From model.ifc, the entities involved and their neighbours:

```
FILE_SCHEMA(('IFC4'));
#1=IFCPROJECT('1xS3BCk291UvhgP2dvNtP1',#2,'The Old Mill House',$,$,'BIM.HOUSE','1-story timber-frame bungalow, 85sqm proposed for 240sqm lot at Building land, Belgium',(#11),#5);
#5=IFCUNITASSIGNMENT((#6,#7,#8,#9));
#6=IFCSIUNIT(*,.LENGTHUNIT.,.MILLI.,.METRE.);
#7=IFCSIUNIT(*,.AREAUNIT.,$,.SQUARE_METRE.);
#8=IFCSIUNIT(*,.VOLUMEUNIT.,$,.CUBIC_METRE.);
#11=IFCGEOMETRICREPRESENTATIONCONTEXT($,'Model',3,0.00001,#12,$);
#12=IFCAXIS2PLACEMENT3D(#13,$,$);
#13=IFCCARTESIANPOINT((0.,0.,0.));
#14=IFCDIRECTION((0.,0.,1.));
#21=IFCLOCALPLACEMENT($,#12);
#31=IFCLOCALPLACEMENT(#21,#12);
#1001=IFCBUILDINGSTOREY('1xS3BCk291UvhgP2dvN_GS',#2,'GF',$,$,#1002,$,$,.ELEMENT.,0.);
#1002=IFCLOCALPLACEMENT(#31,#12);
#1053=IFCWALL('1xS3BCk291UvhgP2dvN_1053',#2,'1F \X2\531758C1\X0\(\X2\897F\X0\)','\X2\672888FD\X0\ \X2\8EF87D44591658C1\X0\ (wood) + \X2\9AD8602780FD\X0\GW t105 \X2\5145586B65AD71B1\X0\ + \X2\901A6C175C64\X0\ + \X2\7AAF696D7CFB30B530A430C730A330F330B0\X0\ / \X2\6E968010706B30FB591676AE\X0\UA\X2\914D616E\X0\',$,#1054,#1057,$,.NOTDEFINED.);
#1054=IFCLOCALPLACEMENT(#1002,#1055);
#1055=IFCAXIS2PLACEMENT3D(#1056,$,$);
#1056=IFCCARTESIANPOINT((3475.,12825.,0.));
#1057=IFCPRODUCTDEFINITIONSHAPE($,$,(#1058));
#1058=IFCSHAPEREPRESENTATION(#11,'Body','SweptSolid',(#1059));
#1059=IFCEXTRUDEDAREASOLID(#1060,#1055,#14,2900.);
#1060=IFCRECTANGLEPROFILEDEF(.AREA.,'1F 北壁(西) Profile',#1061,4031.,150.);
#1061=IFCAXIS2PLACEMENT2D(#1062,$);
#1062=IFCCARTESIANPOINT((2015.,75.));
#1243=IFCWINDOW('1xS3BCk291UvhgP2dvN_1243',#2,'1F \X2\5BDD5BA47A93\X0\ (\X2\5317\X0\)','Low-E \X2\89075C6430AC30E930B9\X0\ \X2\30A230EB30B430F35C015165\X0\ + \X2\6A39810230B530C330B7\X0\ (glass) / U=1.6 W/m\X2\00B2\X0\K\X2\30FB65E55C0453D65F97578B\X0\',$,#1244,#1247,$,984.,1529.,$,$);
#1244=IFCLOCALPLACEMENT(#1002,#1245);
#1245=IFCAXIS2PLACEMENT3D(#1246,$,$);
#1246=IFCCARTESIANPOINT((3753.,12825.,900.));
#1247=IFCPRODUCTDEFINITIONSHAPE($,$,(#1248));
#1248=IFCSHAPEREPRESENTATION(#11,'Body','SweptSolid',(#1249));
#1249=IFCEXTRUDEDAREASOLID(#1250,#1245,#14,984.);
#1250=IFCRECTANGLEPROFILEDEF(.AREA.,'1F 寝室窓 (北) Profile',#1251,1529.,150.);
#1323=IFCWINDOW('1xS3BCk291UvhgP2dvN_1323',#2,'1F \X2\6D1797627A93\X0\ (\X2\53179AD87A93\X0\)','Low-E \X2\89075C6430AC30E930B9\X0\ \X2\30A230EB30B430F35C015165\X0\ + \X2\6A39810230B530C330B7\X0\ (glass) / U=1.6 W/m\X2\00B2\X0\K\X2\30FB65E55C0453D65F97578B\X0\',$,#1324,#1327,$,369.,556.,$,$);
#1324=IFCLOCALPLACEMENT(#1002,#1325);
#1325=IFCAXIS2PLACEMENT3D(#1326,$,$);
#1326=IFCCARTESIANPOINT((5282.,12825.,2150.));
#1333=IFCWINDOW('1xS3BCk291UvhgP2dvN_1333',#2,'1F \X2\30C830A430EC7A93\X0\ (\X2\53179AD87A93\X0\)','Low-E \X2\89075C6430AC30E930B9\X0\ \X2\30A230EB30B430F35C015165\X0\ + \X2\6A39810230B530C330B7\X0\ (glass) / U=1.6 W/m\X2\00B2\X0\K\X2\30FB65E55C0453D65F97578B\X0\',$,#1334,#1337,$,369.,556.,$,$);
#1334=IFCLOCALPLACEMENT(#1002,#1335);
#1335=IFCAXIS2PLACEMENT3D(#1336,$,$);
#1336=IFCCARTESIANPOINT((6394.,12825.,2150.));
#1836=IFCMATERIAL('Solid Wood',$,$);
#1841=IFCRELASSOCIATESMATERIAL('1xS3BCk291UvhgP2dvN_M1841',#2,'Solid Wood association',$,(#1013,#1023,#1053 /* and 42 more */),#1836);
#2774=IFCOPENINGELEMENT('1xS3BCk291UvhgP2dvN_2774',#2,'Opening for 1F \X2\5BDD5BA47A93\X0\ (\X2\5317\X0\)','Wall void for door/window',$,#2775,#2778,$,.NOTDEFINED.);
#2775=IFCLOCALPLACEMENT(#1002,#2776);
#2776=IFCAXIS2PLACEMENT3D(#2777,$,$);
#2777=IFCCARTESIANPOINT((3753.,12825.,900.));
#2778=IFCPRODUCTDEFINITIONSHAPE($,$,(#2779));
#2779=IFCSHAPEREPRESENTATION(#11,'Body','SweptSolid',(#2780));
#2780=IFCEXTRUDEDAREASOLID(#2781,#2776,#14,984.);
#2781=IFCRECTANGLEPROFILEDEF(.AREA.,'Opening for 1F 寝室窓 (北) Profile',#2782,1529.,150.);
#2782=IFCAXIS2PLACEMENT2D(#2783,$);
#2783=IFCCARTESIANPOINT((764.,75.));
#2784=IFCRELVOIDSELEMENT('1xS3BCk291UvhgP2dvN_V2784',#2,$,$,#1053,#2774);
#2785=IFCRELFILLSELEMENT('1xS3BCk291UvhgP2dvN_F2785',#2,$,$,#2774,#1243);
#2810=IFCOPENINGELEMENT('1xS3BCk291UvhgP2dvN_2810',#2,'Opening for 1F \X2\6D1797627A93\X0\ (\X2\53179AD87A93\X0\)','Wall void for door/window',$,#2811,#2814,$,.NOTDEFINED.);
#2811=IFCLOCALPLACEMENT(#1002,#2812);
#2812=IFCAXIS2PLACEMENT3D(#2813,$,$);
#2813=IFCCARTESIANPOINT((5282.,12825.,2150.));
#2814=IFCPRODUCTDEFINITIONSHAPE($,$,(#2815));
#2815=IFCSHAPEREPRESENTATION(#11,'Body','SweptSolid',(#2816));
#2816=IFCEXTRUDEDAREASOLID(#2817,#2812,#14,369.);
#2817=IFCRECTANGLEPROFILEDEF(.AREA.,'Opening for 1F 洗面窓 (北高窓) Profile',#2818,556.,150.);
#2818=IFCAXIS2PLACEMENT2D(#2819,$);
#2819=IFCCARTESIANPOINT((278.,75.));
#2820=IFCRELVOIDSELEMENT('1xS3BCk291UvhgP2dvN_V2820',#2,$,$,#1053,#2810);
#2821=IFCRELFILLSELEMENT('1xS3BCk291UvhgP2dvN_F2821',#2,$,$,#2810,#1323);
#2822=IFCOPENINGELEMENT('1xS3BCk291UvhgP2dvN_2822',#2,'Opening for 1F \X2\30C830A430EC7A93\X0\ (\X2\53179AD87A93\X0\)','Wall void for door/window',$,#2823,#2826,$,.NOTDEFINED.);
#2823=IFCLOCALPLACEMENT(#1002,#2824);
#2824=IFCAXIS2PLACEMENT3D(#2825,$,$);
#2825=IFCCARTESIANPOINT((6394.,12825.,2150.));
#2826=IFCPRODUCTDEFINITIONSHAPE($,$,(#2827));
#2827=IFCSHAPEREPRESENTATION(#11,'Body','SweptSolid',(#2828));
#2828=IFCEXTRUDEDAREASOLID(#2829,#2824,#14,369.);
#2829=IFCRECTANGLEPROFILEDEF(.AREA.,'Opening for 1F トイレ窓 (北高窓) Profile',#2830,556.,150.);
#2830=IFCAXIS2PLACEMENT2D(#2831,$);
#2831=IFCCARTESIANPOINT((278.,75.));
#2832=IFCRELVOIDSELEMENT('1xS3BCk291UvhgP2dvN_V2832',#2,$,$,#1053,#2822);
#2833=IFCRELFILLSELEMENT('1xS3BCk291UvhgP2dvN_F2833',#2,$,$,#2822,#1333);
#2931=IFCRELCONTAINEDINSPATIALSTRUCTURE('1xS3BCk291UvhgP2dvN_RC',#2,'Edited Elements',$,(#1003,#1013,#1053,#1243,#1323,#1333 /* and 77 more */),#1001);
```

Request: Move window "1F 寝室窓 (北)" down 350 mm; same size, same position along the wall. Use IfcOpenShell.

```python
import numpy as np
import ifcopenshell
import ifcopenshell.api.geometry
import ifcopenshell.util.placement
import ifcopenshell.util.unit

model = ifcopenshell.open("model.ifc")
unit_scale = ifcopenshell.util.unit.calculate_unit_scale(model)

window = model.by_id(1243)
opening = window.FillsVoids[0].RelatingOpeningElement
dz = -0.35 / unit_scale

shift = np.array([0.0, 0.0, dz])
# The window is not placed relative to its opening, so move both.
for product in (opening, window):
    matrix = ifcopenshell.util.placement.get_local_placement(product.ObjectPlacement)
    matrix[:3, 3] += shift
    ifcopenshell.api.geometry.edit_object_placement(model, product=product, matrix=matrix, is_si=False)

print(f"moved by {dz * unit_scale:+.3f} m")

model.write("model_updated.ifc")
```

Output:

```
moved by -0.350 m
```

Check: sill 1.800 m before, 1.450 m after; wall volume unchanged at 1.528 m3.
